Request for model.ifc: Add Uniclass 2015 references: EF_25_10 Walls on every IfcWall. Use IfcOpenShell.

First a look at what the model holds.

```python
import ifcopenshell

model = ifcopenshell.open("model.ifc")
print(model.schema)
print("classifications:", [c.Name for c in model.by_type("IfcClassification")])
for ifc_class in ("IfcDoor", "IfcRoof", "IfcStair", "IfcWall", "IfcWindow"):
    print(ifc_class, len(model.by_type(ifc_class)))
```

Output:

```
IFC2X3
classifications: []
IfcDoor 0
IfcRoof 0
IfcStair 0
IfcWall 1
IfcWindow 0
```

```python
import ifcopenshell
import ifcopenshell.api.classification

model = ifcopenshell.open("model.ifc")

# IFC2X3 requires Source and Edition and has no link from the project to the system.
system = model.create_entity("IfcClassification", Source="NBS", Edition="2015", Name="Uniclass 2015")

codes = {
    "IfcWall": ("EF_25_10", "Walls"),
}
for ifc_class, (code, name) in codes.items():
    products = model.by_type(ifc_class)
    ifcopenshell.api.classification.add_reference(
        model, products=products, classification=system, identification=code, name=name
    )
    print(code, len(products))

model.write("model_edited.ifc")
```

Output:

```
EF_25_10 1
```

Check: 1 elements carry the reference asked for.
